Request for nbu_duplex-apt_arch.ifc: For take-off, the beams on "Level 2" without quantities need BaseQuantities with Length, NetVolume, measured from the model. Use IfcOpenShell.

First a look at what the model holds.

```python
import ifcopenshell
import ifcopenshell.util.element
import ifcopenshell.util.unit

model = ifcopenshell.open("nbu_duplex-apt_arch.ifc")
print(model.schema)
for unit_type in ("LENGTHUNIT", "AREAUNIT", "VOLUMEUNIT"):
    print(unit_type, ifcopenshell.util.unit.calculate_unit_scale(model, unit_type))
storey = next(s for s in model.by_type("IfcBuildingStorey") if s.Name == "Level 2")
beams = [e for e in ifcopenshell.util.element.get_decomposition(storey) if e.is_a("IfcBeam")]
for e in sorted(beams, key=lambda e: e.id()):
    print(e.id(), e.is_a(), e.Name, list(ifcopenshell.util.element.get_psets(e, qtos_only=True)), sep=" | ")
```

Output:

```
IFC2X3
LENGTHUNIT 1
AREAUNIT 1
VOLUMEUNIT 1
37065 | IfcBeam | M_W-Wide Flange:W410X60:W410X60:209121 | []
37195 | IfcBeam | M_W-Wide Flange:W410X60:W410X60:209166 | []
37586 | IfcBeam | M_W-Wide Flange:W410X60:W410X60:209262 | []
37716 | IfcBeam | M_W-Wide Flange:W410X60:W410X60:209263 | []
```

```python
import ifcopenshell
import ifcopenshell.api.pset
import ifcopenshell.geom
import ifcopenshell.util.element
import ifcopenshell.util.shape
import ifcopenshell.util.unit

model = ifcopenshell.open("nbu_duplex-apt_arch.ifc")
unit_scale = ifcopenshell.util.unit.calculate_unit_scale(model)
volume_scale = ifcopenshell.util.unit.calculate_unit_scale(model, "VOLUMEUNIT")
settings = ifcopenshell.geom.settings()

storey = next(s for s in model.by_type("IfcBuildingStorey") if s.Name == "Level 2")
beams = [e for e in ifcopenshell.util.element.get_decomposition(storey) if e.is_a("IfcBeam")]

for e in sorted(beams, key=lambda e: e.id()):
    if ifcopenshell.util.element.get_psets(e, qtos_only=True, should_inherit=False):
        continue
    # Geometry comes back in metres, in the element's own axes.
    shape = ifcopenshell.geom.create_shape(settings, e)
    values = {
        "Length": ifcopenshell.util.shape.get_max_xyz(shape.geometry) / unit_scale,
        "NetVolume": ifcopenshell.util.shape.get_volume(shape.geometry) / volume_scale,
    }
    qto = ifcopenshell.api.pset.add_qto(model, product=e, name="BaseQuantities")
    ifcopenshell.api.pset.edit_qto(model, qto=qto, properties=values)
    print(e.id(), {k: round(v, 3) for k, v in values.items()})

model.write("nbu_duplex-apt_arch_v2.ifc")
```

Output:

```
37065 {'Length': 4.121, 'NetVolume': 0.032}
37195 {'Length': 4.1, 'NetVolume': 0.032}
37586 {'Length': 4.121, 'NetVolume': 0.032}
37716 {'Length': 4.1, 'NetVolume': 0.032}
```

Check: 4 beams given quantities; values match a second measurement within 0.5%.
